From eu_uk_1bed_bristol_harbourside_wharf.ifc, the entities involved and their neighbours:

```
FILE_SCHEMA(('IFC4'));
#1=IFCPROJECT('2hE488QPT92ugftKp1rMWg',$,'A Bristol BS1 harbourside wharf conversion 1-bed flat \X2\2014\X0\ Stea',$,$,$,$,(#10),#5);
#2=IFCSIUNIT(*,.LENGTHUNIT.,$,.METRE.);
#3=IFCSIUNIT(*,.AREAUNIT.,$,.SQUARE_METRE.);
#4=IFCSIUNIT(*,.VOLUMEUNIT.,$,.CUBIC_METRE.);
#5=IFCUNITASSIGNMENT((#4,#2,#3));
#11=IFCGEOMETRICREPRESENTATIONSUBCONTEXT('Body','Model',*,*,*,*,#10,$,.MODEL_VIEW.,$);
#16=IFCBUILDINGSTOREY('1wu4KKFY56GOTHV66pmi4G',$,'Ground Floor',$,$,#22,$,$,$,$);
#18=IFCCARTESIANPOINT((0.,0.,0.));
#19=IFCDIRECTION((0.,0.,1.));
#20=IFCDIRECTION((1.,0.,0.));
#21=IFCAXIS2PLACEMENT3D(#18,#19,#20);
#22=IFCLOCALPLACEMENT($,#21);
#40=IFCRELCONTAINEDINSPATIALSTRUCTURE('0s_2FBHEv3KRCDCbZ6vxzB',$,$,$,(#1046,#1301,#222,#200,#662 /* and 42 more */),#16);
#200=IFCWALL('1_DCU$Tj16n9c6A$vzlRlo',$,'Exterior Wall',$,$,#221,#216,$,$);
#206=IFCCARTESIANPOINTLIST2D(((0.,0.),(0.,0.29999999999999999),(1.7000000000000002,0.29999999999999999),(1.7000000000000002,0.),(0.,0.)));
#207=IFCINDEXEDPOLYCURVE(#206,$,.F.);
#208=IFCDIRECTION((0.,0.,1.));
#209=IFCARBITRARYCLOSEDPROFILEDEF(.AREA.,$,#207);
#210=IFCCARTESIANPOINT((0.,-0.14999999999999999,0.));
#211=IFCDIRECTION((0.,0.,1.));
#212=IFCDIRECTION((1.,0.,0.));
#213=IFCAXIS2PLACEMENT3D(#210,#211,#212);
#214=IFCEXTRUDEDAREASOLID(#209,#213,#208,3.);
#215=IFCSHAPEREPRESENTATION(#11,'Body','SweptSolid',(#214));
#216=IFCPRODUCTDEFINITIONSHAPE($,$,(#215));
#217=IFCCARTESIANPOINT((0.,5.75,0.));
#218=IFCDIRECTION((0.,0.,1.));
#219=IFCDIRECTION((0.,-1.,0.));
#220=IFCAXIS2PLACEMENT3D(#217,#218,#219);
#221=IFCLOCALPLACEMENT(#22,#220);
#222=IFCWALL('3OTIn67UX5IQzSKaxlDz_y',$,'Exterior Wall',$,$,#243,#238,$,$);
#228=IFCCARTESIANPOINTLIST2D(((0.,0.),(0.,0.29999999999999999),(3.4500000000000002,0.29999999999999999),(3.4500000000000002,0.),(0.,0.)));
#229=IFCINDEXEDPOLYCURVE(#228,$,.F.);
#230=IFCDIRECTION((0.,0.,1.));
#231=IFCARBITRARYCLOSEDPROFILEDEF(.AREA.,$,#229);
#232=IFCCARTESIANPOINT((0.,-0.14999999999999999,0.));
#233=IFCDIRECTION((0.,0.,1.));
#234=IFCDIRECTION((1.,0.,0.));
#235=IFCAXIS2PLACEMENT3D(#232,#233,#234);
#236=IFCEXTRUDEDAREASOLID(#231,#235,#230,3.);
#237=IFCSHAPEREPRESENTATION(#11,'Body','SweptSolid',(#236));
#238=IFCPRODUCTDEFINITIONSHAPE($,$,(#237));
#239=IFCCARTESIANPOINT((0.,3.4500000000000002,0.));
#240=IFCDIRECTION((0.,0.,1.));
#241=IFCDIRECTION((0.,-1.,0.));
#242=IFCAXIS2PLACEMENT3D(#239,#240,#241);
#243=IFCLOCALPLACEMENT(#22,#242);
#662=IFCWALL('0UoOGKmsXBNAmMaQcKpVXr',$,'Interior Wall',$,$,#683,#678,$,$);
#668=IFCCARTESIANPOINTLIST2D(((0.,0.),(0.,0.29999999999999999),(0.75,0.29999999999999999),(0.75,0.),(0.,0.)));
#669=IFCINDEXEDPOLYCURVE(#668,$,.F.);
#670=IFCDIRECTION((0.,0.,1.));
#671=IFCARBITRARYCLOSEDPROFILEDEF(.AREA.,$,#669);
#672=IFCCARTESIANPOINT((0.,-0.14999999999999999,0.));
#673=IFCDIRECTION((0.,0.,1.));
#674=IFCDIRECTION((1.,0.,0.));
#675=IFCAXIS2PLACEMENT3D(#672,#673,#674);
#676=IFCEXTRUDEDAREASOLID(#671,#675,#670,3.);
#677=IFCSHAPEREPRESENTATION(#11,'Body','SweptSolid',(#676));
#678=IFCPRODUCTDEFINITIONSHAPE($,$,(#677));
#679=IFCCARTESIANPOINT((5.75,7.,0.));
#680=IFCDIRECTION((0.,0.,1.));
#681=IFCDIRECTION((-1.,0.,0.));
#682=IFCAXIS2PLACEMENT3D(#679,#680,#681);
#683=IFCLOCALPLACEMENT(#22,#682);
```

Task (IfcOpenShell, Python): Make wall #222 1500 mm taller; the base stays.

```python
import ifcopenshell
import ifcopenshell.geom
import ifcopenshell.util.representation
import ifcopenshell.util.shape

model = ifcopenshell.open("eu_uk_1bed_bristol_harbourside_wharf.ifc")
settings = ifcopenshell.geom.settings()


def volume(element):
    """Net volume in cubic metres, openings subtracted."""
    shape = ifcopenshell.geom.create_shape(settings, element)
    return ifcopenshell.util.shape.get_volume(shape.geometry)


wall = model.by_guid("3OTIn67UX5IQzSKaxlDz_y")
before = volume(wall)

body = ifcopenshell.util.representation.get_representation(wall, "Model", "Body")
solid = body.Items[0]
old_height = solid.Depth
solid.Depth += 1.5
after = volume(wall)

print(f"height {old_height:g} -> {solid.Depth:g}, volume {before:.3f} -> {after:.3f} m3")

model.write("eu_uk_1bed_bristol_harbourside_wharf-out.ifc")
```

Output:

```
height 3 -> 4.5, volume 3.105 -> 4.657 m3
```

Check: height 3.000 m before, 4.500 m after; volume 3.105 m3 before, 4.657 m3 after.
